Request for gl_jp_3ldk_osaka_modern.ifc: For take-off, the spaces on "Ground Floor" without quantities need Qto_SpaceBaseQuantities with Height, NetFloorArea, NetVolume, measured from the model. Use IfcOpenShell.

First a look at what the model holds.

```python
import ifcopenshell
import ifcopenshell.util.element
import ifcopenshell.util.unit

model = ifcopenshell.open("gl_jp_3ldk_osaka_modern.ifc")
print(model.schema)
for unit_type in ("LENGTHUNIT", "AREAUNIT", "VOLUMEUNIT"):
    print(unit_type, ifcopenshell.util.unit.calculate_unit_scale(model, unit_type))
storey = next(s for s in model.by_type("IfcBuildingStorey") if s.Name == "Ground Floor")
spaces = [e for e in ifcopenshell.util.element.get_decomposition(storey) if e.is_a("IfcSpace")]
for e in sorted(spaces, key=lambda e: e.id()):
    print(e.id(), e.is_a(), e.Name, list(ifcopenshell.util.element.get_psets(e, qtos_only=True)), sep=" | ")
```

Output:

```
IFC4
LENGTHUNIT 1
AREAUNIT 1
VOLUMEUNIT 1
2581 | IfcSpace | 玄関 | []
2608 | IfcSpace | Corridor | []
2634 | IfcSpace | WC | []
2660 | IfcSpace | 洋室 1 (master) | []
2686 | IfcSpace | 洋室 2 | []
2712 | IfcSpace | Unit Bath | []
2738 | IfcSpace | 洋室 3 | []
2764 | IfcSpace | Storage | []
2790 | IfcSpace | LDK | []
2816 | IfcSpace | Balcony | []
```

```python
import ifcopenshell
import ifcopenshell.api.pset
import ifcopenshell.geom
import ifcopenshell.util.element
import ifcopenshell.util.shape
import ifcopenshell.util.unit

model = ifcopenshell.open("gl_jp_3ldk_osaka_modern.ifc")
unit_scale = ifcopenshell.util.unit.calculate_unit_scale(model)
area_scale = ifcopenshell.util.unit.calculate_unit_scale(model, "AREAUNIT")
volume_scale = ifcopenshell.util.unit.calculate_unit_scale(model, "VOLUMEUNIT")
settings = ifcopenshell.geom.settings()

storey = next(s for s in model.by_type("IfcBuildingStorey") if s.Name == "Ground Floor")
spaces = [e for e in ifcopenshell.util.element.get_decomposition(storey) if e.is_a("IfcSpace")]

for e in sorted(spaces, key=lambda e: e.id()):
    if ifcopenshell.util.element.get_psets(e, qtos_only=True, should_inherit=False):
        continue
    # Geometry comes back in metres, in the element's own axes.
    shape = ifcopenshell.geom.create_shape(settings, e)
    values = {
        "Height": ifcopenshell.util.shape.get_z(shape.geometry) / unit_scale,
        "NetFloorArea": ifcopenshell.util.shape.get_footprint_area(shape.geometry) / area_scale,
        "NetVolume": ifcopenshell.util.shape.get_volume(shape.geometry) / volume_scale,
    }
    qto = ifcopenshell.api.pset.add_qto(model, product=e, name="Qto_SpaceBaseQuantities")
    ifcopenshell.api.pset.edit_qto(model, qto=qto, properties=values)
    print(e.id(), {k: round(v, 3) for k, v in values.items()})

model.write("gl_jp_3ldk_osaka_modern-out.ifc")
```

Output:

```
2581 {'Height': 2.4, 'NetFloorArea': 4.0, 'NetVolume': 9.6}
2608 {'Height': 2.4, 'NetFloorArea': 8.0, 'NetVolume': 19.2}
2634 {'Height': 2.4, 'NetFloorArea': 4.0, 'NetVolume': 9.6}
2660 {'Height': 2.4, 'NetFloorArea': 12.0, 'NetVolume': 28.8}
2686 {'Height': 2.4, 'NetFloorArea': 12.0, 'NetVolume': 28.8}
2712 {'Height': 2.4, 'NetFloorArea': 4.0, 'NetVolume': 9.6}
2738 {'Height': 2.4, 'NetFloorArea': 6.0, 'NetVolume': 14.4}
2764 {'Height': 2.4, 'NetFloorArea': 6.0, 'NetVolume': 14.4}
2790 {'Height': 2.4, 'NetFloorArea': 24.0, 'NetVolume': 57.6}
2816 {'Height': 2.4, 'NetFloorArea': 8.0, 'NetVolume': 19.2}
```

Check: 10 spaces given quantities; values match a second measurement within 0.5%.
